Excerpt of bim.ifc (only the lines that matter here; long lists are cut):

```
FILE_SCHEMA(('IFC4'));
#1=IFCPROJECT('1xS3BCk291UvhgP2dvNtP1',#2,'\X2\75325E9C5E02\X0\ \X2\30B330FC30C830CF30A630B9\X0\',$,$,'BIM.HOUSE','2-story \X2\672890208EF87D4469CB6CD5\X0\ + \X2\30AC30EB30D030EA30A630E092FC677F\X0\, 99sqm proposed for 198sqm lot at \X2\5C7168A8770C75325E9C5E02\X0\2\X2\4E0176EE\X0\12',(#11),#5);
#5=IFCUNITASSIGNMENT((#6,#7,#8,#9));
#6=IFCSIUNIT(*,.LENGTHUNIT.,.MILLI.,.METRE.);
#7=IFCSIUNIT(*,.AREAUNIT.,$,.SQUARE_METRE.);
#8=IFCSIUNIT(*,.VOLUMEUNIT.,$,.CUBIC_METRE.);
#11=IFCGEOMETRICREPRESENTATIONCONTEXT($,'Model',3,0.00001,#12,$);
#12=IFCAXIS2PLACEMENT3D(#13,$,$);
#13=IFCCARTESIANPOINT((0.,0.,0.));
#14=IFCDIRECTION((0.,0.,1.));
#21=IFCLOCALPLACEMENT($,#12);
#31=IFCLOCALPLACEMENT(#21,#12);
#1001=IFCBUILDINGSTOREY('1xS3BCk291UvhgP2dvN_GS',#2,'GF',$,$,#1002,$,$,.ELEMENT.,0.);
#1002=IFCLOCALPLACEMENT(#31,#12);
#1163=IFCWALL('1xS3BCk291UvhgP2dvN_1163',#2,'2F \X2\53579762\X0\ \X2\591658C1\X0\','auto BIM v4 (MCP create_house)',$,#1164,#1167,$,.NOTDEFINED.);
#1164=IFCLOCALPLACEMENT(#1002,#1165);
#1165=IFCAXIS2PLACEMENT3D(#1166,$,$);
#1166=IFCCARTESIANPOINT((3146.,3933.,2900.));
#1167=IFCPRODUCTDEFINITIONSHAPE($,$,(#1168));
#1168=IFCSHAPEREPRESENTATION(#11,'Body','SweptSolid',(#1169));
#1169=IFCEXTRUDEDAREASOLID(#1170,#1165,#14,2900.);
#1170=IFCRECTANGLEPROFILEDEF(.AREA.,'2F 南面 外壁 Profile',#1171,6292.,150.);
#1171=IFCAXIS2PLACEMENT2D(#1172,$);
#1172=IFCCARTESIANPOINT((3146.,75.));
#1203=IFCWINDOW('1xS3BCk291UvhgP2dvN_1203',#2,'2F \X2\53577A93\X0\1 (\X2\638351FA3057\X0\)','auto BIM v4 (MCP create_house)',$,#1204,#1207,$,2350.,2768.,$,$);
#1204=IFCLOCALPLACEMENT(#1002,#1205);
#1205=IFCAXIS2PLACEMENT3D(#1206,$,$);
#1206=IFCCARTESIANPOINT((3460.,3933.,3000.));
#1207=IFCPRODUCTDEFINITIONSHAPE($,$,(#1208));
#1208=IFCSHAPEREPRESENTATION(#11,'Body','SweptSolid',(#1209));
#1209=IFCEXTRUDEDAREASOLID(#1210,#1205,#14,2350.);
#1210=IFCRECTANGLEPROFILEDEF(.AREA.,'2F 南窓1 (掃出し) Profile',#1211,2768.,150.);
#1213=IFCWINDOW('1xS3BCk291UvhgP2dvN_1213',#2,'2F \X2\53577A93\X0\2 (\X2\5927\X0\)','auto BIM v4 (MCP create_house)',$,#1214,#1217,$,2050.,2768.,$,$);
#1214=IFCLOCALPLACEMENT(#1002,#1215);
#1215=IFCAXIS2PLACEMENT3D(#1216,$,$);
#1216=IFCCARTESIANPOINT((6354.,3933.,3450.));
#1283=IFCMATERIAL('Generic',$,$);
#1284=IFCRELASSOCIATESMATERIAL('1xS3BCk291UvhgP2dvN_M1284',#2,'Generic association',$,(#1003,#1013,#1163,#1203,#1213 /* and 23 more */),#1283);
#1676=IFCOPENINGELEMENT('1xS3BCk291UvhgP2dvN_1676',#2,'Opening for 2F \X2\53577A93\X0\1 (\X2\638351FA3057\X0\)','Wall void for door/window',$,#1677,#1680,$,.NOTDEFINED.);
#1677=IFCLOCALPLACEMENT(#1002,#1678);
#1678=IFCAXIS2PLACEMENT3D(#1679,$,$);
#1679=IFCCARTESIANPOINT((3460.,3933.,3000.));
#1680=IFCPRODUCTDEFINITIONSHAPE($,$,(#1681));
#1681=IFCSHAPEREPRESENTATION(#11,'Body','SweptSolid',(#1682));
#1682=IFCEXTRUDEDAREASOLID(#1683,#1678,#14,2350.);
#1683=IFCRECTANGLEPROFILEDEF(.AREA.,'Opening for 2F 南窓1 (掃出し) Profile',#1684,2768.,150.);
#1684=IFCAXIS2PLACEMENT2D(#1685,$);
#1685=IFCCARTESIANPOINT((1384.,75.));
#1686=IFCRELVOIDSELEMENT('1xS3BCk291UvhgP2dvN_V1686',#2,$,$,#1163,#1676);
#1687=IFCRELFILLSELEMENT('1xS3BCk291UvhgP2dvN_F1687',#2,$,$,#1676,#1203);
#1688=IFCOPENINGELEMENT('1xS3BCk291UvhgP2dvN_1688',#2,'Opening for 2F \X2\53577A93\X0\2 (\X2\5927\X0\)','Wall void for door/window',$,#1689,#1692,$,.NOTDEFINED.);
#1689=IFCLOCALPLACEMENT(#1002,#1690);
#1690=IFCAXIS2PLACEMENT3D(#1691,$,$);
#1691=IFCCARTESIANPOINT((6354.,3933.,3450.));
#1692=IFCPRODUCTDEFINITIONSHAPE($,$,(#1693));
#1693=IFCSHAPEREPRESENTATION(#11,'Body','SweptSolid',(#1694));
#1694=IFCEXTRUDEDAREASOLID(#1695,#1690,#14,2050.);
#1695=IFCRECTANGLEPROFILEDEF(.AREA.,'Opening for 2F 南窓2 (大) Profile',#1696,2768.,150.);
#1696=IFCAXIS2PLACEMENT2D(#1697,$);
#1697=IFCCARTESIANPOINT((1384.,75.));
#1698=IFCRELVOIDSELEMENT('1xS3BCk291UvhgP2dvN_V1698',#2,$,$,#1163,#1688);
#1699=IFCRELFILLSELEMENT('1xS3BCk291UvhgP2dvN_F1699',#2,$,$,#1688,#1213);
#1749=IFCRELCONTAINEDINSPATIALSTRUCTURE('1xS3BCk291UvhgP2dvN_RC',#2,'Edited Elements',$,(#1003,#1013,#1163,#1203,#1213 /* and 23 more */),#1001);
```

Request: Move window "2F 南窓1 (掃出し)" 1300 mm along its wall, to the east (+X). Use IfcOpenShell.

```python
import ifcopenshell
import ifcopenshell.api.geometry
import ifcopenshell.util.placement
import ifcopenshell.util.unit

model = ifcopenshell.open("bim.ifc")
unit_scale = ifcopenshell.util.unit.calculate_unit_scale(model)

window = model.by_guid("1xS3BCk291UvhgP2dvN_1203")
opening = window.FillsVoids[0].RelatingOpeningElement
wall = opening.VoidsElements[0].RelatingBuildingElement

wall_matrix = ifcopenshell.util.placement.get_local_placement(wall.ObjectPlacement)
shift = wall_matrix[:3, 0] * 1.3 / unit_scale
before = ifcopenshell.util.placement.get_local_placement(window.ObjectPlacement)[:3, 3].copy()

# The window is not placed relative to its opening, so move both.
for product in (opening, window):
    matrix = ifcopenshell.util.placement.get_local_placement(product.ObjectPlacement)
    matrix[:3, 3] += shift
    ifcopenshell.api.geometry.edit_object_placement(model, product=product, matrix=matrix, is_si=False)

after = ifcopenshell.util.placement.get_local_placement(window.ObjectPlacement)[:3, 3]
print("window moved by", (after - before).round(3) + 0.0)

model.write("bim_rev.ifc")
```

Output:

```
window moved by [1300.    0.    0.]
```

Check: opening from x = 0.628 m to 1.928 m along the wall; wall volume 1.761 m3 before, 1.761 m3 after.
